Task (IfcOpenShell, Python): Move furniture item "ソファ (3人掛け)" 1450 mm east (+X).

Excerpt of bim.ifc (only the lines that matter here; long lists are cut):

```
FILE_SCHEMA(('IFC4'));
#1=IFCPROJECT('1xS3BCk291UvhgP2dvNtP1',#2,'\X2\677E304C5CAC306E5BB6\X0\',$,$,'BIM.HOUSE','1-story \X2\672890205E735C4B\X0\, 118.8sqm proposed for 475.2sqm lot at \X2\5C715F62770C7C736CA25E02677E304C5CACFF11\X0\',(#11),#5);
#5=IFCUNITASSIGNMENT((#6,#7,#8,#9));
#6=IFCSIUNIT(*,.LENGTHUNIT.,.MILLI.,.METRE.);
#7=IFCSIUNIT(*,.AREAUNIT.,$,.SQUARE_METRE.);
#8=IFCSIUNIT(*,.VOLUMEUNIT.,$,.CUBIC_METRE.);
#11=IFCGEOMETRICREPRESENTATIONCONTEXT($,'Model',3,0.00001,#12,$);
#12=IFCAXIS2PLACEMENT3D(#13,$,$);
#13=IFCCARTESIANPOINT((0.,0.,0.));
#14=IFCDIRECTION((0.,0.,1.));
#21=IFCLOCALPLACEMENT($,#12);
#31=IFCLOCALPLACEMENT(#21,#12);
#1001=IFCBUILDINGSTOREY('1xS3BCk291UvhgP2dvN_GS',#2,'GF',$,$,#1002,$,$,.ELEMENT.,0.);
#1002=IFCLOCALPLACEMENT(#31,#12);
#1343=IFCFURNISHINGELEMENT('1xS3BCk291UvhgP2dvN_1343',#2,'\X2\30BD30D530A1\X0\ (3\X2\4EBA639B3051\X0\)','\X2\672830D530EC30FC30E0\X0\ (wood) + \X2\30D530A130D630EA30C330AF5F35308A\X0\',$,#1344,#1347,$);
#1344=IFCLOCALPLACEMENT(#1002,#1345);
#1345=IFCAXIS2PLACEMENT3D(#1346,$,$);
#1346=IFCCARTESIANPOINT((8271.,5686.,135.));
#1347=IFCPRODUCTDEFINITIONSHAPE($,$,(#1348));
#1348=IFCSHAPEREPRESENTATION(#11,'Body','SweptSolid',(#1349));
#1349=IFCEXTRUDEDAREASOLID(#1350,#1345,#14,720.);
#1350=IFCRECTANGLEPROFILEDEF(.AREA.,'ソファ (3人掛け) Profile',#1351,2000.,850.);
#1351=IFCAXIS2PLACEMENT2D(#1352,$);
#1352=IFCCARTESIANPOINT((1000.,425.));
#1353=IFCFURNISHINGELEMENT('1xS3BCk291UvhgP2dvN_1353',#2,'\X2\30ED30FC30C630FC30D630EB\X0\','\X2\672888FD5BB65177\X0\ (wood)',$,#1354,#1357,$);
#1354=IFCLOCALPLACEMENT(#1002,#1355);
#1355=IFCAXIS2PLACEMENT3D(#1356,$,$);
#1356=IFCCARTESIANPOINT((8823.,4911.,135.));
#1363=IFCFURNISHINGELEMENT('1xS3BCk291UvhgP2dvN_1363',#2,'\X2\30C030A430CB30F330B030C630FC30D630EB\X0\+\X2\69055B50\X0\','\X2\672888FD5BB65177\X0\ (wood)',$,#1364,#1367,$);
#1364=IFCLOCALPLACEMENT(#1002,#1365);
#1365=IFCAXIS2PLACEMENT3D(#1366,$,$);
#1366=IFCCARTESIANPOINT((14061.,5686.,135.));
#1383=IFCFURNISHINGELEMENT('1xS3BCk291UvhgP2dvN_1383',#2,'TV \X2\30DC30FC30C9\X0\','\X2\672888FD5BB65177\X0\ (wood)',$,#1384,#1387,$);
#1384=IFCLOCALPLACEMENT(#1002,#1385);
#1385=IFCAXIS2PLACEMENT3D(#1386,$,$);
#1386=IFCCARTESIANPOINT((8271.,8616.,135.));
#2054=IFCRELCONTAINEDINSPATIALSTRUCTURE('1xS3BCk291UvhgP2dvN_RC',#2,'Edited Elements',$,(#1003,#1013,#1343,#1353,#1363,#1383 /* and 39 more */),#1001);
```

```python
import ifcopenshell
import ifcopenshell.api.geometry
import ifcopenshell.util.placement

model = ifcopenshell.open("bim.ifc")

item = model.by_id(1343)
matrix = ifcopenshell.util.placement.get_local_placement(item.ObjectPlacement)
matrix[0, 3] += 1450.0
ifcopenshell.api.geometry.edit_object_placement(model, product=item, matrix=matrix, is_si=False)

print(ifcopenshell.util.placement.get_local_placement(item.ObjectPlacement).round(3) + 0.0)

model.write("bim-out.ifc")
```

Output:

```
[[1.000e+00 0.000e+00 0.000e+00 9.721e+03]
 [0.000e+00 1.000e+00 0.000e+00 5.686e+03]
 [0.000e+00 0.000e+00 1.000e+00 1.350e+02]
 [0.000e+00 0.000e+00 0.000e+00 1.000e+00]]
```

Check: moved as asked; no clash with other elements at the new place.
